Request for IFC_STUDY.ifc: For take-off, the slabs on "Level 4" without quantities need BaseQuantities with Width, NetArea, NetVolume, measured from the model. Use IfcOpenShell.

First a look at what the model holds.

```python
import ifcopenshell
import ifcopenshell.util.element
import ifcopenshell.util.unit

model = ifcopenshell.open("IFC_STUDY.ifc")
print(model.schema)
for unit_type in ("LENGTHUNIT", "AREAUNIT", "VOLUMEUNIT"):
    print(unit_type, ifcopenshell.util.unit.calculate_unit_scale(model, unit_type))
storey = next(s for s in model.by_type("IfcBuildingStorey") if s.Name == "Level 4")
slabs = [e for e in ifcopenshell.util.element.get_decomposition(storey) if e.is_a("IfcSlab")]
for e in sorted(slabs, key=lambda e: e.id()):
    print(e.id(), e.is_a(), e.Name, list(ifcopenshell.util.element.get_psets(e, qtos_only=True)), sep=" | ")
```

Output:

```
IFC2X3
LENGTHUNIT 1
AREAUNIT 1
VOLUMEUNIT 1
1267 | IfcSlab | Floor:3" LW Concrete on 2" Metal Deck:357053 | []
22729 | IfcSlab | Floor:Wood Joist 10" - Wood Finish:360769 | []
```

```python
import ifcopenshell
import ifcopenshell.api.pset
import ifcopenshell.geom
import ifcopenshell.util.element
import ifcopenshell.util.shape
import ifcopenshell.util.unit

model = ifcopenshell.open("IFC_STUDY.ifc")
unit_scale = ifcopenshell.util.unit.calculate_unit_scale(model)
area_scale = ifcopenshell.util.unit.calculate_unit_scale(model, "AREAUNIT")
volume_scale = ifcopenshell.util.unit.calculate_unit_scale(model, "VOLUMEUNIT")
settings = ifcopenshell.geom.settings()

storey = next(s for s in model.by_type("IfcBuildingStorey") if s.Name == "Level 4")
slabs = [e for e in ifcopenshell.util.element.get_decomposition(storey) if e.is_a("IfcSlab")]

for e in sorted(slabs, key=lambda e: e.id()):
    if ifcopenshell.util.element.get_psets(e, qtos_only=True, should_inherit=False):
        continue
    # Geometry comes back in metres, in the element's own axes.
    shape = ifcopenshell.geom.create_shape(settings, e)
    values = {
        "Width": ifcopenshell.util.shape.get_z(shape.geometry) / unit_scale,
        "NetArea": ifcopenshell.util.shape.get_footprint_area(shape.geometry) / area_scale,
        "NetVolume": ifcopenshell.util.shape.get_volume(shape.geometry) / volume_scale,
    }
    qto = ifcopenshell.api.pset.add_qto(model, product=e, name="BaseQuantities")
    ifcopenshell.api.pset.edit_qto(model, qto=qto, properties=values)
    print(e.id(), {k: round(v, 3) for k, v in values.items()})

model.write("IFC_STUDY_v2.ifc")
```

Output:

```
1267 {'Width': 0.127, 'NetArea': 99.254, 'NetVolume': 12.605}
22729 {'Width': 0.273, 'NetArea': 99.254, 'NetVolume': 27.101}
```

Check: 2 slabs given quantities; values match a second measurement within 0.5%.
